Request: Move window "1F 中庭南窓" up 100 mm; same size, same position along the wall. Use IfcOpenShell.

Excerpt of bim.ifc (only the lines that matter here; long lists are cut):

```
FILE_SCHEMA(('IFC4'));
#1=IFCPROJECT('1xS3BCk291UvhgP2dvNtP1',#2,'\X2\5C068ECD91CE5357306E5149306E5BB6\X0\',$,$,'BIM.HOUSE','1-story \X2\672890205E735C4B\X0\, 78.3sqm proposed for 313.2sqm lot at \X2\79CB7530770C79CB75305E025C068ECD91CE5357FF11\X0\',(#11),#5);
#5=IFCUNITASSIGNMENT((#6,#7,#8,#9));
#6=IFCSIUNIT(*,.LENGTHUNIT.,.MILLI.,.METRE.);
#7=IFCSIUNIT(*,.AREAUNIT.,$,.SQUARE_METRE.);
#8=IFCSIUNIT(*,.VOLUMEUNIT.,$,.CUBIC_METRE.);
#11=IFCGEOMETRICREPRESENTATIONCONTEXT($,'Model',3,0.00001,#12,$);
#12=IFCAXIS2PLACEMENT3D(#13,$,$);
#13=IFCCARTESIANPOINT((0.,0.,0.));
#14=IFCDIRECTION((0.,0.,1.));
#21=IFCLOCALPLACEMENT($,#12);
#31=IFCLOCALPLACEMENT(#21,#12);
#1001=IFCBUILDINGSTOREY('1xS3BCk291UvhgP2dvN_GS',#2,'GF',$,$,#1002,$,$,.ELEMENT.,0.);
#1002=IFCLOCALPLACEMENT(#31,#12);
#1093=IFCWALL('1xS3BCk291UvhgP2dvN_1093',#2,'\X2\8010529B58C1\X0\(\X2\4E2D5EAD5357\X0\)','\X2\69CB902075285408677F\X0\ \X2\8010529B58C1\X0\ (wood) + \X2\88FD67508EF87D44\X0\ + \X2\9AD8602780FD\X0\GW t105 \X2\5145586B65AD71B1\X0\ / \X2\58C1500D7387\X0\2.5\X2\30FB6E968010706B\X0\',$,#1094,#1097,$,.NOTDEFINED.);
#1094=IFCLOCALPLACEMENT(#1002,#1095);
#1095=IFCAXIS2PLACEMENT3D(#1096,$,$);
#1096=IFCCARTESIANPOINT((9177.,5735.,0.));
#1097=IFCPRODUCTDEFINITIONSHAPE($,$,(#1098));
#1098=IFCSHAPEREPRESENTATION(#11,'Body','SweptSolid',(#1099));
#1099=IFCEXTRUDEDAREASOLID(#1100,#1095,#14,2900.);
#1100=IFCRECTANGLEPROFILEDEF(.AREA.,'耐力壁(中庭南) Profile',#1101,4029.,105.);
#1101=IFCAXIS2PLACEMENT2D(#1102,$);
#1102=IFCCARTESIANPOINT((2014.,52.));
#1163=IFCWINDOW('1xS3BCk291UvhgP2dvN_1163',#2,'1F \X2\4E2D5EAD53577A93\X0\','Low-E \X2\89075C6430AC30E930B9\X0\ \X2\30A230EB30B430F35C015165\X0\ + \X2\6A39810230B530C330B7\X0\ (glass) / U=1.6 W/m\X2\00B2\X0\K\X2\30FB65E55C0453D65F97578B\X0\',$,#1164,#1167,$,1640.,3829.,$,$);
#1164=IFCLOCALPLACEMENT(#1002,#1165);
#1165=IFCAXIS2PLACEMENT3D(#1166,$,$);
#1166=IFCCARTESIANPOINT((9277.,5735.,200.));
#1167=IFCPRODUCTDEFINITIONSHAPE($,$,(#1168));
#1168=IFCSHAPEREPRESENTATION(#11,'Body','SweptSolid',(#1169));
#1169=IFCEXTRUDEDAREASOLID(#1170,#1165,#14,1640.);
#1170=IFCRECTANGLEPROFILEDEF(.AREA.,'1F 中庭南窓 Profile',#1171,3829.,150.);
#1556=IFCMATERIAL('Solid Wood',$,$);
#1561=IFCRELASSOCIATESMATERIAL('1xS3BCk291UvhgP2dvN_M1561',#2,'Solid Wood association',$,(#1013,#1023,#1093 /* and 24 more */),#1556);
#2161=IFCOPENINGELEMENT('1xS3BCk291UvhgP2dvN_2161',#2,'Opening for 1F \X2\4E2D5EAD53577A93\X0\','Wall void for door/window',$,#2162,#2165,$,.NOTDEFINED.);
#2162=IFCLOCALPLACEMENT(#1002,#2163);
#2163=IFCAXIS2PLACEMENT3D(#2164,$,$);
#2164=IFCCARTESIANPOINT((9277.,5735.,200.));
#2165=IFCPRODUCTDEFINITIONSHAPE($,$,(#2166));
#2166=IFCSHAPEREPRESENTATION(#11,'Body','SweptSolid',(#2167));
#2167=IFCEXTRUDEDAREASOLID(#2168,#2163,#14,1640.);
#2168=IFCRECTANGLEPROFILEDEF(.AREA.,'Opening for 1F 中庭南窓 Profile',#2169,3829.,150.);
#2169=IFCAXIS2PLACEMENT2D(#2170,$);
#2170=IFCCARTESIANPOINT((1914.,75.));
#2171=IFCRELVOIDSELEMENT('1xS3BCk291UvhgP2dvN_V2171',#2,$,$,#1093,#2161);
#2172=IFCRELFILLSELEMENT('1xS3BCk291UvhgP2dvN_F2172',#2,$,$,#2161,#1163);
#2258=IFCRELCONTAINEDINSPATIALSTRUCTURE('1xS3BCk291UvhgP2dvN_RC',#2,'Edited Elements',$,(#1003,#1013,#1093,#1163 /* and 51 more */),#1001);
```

```python
import numpy as np
import ifcopenshell
import ifcopenshell.api.geometry
import ifcopenshell.util.placement
import ifcopenshell.util.unit

model = ifcopenshell.open("bim.ifc")
unit_scale = ifcopenshell.util.unit.calculate_unit_scale(model)

window = model.by_guid("1xS3BCk291UvhgP2dvN_1163")
opening = window.FillsVoids[0].RelatingOpeningElement
dz = 0.1 / unit_scale

shift = np.array([0.0, 0.0, dz])
# The window is not placed relative to its opening, so move both.
for product in (opening, window):
    matrix = ifcopenshell.util.placement.get_local_placement(product.ObjectPlacement)
    matrix[:3, 3] += shift
    ifcopenshell.api.geometry.edit_object_placement(model, product=product, matrix=matrix, is_si=False)

print(f"moved by {dz * unit_scale:+.3f} m")

model.write("bim_v2.ifc")
```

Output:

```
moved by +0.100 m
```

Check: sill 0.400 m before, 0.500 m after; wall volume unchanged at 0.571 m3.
